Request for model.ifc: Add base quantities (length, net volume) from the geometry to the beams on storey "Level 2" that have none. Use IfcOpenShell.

First a look at what the model holds.

```python
import ifcopenshell
import ifcopenshell.util.element
import ifcopenshell.util.unit

model = ifcopenshell.open("model.ifc")
print(model.schema)
for unit_type in ("LENGTHUNIT", "AREAUNIT", "VOLUMEUNIT"):
    print(unit_type, ifcopenshell.util.unit.calculate_unit_scale(model, unit_type))
storey = next(s for s in model.by_type("IfcBuildingStorey") if s.Name == "Level 2")
beams = [e for e in ifcopenshell.util.element.get_decomposition(storey) if e.is_a("IfcBeam")]
for e in sorted(beams, key=lambda e: e.id()):
    print(e.id(), e.is_a(), e.Name, list(ifcopenshell.util.element.get_psets(e, qtos_only=True)), sep=" | ")
```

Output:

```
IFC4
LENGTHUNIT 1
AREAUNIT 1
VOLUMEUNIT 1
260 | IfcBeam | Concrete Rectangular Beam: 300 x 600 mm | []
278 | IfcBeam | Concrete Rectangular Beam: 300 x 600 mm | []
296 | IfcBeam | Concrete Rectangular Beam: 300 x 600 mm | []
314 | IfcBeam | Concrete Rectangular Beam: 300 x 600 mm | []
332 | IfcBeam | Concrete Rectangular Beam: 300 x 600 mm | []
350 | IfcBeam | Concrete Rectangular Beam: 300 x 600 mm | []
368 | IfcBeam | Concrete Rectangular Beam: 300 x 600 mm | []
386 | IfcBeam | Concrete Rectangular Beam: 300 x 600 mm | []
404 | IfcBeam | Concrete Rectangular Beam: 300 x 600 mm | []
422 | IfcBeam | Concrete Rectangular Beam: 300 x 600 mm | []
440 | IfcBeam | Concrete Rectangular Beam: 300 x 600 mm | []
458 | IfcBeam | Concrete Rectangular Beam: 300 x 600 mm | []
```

```python
import ifcopenshell
import ifcopenshell.api.pset
import ifcopenshell.geom
import ifcopenshell.util.element
import ifcopenshell.util.shape
import ifcopenshell.util.unit

model = ifcopenshell.open("model.ifc")
unit_scale = ifcopenshell.util.unit.calculate_unit_scale(model)
volume_scale = ifcopenshell.util.unit.calculate_unit_scale(model, "VOLUMEUNIT")
settings = ifcopenshell.geom.settings()

storey = next(s for s in model.by_type("IfcBuildingStorey") if s.Name == "Level 2")
beams = [e for e in ifcopenshell.util.element.get_decomposition(storey) if e.is_a("IfcBeam")]

for e in sorted(beams, key=lambda e: e.id()):
    if ifcopenshell.util.element.get_psets(e, qtos_only=True, should_inherit=False):
        continue
    # Geometry comes back in metres, in the element's own axes.
    shape = ifcopenshell.geom.create_shape(settings, e)
    values = {
        "Length": ifcopenshell.util.shape.get_max_xyz(shape.geometry) / unit_scale,
        "NetVolume": ifcopenshell.util.shape.get_volume(shape.geometry) / volume_scale,
    }
    qto = ifcopenshell.api.pset.add_qto(model, product=e, name="Qto_BeamBaseQuantities")
    ifcopenshell.api.pset.edit_qto(model, qto=qto, properties=values)
    print(e.id(), {k: round(v, 3) for k, v in values.items()})

model.write("model_edited.ifc")
```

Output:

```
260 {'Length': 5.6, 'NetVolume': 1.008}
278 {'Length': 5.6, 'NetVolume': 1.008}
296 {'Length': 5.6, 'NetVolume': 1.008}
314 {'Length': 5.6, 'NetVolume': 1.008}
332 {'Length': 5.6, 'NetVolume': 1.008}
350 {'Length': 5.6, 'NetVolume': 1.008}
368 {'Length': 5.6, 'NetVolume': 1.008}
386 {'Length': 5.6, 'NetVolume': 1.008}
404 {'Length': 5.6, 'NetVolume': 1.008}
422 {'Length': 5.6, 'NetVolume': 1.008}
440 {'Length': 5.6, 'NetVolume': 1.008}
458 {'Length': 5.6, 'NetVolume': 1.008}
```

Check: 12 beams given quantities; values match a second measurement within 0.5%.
